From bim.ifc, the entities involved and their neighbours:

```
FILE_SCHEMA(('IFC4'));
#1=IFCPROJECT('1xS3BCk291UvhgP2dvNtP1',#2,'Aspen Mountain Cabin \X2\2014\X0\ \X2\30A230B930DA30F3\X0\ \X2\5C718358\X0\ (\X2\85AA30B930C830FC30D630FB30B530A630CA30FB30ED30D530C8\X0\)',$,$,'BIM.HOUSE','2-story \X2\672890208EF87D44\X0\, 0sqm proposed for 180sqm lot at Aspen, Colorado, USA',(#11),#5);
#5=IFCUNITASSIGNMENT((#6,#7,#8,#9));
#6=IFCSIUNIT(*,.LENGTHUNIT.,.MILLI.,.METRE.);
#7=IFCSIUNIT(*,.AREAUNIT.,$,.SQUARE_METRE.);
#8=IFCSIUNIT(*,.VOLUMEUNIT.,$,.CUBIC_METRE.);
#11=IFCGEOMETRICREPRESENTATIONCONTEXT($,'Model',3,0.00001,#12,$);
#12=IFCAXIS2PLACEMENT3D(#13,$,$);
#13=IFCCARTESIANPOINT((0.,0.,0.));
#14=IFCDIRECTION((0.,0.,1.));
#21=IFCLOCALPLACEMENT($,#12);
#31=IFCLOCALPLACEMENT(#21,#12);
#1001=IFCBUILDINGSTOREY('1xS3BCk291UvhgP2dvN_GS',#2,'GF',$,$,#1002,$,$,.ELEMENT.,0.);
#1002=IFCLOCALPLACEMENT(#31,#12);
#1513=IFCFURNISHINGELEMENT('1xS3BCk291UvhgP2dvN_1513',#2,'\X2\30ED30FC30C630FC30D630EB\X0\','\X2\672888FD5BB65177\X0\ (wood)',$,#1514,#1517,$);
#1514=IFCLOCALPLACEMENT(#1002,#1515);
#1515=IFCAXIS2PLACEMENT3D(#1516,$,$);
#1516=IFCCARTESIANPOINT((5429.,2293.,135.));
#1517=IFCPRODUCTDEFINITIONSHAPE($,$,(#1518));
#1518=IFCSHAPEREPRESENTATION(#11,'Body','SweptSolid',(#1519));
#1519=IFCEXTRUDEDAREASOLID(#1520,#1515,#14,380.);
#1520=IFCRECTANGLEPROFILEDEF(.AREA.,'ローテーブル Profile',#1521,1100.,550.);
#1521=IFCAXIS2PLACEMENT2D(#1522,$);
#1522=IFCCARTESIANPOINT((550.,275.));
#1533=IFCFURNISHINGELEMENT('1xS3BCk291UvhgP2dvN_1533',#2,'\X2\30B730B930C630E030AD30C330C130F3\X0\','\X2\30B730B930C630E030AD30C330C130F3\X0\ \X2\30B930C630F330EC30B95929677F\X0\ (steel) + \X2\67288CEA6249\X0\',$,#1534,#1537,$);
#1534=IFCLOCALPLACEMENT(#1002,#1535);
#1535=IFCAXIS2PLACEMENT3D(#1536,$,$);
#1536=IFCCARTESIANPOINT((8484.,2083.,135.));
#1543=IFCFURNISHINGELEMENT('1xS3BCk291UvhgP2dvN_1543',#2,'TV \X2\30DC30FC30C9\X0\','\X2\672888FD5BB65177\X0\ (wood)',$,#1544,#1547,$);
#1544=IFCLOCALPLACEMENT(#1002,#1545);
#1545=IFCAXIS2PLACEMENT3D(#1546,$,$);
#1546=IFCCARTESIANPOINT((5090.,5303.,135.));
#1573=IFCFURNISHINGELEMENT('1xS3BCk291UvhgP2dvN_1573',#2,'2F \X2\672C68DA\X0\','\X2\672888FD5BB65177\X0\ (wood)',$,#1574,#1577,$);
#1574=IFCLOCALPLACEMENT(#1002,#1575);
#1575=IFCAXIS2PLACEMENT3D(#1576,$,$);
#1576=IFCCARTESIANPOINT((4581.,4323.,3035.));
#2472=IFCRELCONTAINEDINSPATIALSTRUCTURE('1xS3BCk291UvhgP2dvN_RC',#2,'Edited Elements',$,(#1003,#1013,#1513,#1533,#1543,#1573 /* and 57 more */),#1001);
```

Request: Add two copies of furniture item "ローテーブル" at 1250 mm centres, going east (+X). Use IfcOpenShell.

```python
import numpy as np
import ifcopenshell
import ifcopenshell.api.geometry
import ifcopenshell.api.root
import ifcopenshell.util.element
import ifcopenshell.util.placement

model = ifcopenshell.open("bim.ifc")


def reuse_history(source, copy):
    """copy_class also copies each property set's owner history, people and application; keep the originals."""
    for rel in copy.IsDefinedBy:
        if rel.is_a("IfcRelDefinesByProperties") and (history := rel.RelatingPropertyDefinition.OwnerHistory):
            rel.RelatingPropertyDefinition.OwnerHistory = source.OwnerHistory
            ifcopenshell.util.element.remove_deep2(model, history)


source = model.by_id(1513)
base = ifcopenshell.util.placement.get_local_placement(source.ObjectPlacement)
step = np.array([1.0, 0.0, 0.0]) * 1250.0

for i in range(1, 3):
    copy = ifcopenshell.api.root.copy_class(model, product=source)
    copy.Representation = ifcopenshell.util.element.copy_deep(
        model, source.Representation, exclude=["IfcGeometricRepresentationContext", "IfcRepresentationMap"]
    )
    reuse_history(source, copy)
    matrix = base.copy()
    matrix[:3, 3] += i * step
    print("added at", matrix[:3, 3].round(3) + 0.0)
    ifcopenshell.api.geometry.edit_object_placement(model, product=copy, matrix=matrix, is_si=False)

model.write("bim-out.ifc")
```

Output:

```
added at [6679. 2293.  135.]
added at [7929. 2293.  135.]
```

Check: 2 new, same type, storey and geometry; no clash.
